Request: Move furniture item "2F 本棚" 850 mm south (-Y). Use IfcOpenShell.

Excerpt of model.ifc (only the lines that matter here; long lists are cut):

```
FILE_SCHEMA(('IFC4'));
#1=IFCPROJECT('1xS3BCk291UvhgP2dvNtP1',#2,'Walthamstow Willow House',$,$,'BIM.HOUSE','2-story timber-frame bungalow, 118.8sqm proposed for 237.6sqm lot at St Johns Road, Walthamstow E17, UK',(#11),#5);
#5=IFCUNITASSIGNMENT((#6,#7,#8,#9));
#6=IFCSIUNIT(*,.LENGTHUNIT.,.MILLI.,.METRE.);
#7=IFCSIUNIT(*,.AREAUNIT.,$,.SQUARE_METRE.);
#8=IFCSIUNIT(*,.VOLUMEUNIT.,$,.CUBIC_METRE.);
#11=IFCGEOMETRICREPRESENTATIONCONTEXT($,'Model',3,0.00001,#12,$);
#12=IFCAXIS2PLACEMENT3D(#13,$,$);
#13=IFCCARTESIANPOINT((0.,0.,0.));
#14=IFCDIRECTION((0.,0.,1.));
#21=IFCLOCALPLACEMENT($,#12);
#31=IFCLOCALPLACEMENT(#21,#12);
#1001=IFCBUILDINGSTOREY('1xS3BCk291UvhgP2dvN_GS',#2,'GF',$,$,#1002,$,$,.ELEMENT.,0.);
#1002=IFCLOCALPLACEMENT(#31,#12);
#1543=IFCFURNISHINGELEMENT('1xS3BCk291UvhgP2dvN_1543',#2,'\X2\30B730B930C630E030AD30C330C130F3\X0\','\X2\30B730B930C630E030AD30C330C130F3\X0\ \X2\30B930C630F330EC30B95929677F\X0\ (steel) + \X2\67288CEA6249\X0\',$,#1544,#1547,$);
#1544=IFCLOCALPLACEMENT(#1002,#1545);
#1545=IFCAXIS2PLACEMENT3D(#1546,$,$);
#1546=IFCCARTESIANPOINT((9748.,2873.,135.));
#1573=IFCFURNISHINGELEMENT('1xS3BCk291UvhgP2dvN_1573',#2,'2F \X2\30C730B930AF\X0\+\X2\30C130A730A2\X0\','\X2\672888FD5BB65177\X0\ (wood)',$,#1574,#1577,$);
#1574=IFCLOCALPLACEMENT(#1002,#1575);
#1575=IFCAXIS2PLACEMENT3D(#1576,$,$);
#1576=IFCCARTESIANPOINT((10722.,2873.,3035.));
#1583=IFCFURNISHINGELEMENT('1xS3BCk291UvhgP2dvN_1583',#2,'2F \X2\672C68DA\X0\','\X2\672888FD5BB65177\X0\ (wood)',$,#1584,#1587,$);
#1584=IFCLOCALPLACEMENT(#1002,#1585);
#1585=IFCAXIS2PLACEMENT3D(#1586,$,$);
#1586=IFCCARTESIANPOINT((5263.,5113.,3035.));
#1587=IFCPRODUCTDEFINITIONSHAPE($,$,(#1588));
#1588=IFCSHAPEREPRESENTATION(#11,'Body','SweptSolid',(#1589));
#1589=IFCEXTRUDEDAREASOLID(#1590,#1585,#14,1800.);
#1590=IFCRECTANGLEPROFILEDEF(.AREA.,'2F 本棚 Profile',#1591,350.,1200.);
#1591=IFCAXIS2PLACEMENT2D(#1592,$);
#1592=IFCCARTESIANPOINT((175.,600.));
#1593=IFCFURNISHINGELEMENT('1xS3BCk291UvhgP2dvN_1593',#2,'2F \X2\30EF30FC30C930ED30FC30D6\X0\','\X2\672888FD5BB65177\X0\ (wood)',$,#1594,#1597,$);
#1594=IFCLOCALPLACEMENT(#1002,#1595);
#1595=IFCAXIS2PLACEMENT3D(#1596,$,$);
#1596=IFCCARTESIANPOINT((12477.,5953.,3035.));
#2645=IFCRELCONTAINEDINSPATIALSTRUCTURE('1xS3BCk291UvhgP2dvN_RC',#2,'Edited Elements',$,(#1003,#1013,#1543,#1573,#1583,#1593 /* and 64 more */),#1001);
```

```python
import ifcopenshell
import ifcopenshell.api.geometry
import ifcopenshell.util.placement

model = ifcopenshell.open("model.ifc")

item = model.by_id(1583)
matrix = ifcopenshell.util.placement.get_local_placement(item.ObjectPlacement)
matrix[1, 3] -= 850.0
ifcopenshell.api.geometry.edit_object_placement(model, product=item, matrix=matrix, is_si=False)

print(ifcopenshell.util.placement.get_local_placement(item.ObjectPlacement).round(3) + 0.0)

model.write("model-out.ifc")
```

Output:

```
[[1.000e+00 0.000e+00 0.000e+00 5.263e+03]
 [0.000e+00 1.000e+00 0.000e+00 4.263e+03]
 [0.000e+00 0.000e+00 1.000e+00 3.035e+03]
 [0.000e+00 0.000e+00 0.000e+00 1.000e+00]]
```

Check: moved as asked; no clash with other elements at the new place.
